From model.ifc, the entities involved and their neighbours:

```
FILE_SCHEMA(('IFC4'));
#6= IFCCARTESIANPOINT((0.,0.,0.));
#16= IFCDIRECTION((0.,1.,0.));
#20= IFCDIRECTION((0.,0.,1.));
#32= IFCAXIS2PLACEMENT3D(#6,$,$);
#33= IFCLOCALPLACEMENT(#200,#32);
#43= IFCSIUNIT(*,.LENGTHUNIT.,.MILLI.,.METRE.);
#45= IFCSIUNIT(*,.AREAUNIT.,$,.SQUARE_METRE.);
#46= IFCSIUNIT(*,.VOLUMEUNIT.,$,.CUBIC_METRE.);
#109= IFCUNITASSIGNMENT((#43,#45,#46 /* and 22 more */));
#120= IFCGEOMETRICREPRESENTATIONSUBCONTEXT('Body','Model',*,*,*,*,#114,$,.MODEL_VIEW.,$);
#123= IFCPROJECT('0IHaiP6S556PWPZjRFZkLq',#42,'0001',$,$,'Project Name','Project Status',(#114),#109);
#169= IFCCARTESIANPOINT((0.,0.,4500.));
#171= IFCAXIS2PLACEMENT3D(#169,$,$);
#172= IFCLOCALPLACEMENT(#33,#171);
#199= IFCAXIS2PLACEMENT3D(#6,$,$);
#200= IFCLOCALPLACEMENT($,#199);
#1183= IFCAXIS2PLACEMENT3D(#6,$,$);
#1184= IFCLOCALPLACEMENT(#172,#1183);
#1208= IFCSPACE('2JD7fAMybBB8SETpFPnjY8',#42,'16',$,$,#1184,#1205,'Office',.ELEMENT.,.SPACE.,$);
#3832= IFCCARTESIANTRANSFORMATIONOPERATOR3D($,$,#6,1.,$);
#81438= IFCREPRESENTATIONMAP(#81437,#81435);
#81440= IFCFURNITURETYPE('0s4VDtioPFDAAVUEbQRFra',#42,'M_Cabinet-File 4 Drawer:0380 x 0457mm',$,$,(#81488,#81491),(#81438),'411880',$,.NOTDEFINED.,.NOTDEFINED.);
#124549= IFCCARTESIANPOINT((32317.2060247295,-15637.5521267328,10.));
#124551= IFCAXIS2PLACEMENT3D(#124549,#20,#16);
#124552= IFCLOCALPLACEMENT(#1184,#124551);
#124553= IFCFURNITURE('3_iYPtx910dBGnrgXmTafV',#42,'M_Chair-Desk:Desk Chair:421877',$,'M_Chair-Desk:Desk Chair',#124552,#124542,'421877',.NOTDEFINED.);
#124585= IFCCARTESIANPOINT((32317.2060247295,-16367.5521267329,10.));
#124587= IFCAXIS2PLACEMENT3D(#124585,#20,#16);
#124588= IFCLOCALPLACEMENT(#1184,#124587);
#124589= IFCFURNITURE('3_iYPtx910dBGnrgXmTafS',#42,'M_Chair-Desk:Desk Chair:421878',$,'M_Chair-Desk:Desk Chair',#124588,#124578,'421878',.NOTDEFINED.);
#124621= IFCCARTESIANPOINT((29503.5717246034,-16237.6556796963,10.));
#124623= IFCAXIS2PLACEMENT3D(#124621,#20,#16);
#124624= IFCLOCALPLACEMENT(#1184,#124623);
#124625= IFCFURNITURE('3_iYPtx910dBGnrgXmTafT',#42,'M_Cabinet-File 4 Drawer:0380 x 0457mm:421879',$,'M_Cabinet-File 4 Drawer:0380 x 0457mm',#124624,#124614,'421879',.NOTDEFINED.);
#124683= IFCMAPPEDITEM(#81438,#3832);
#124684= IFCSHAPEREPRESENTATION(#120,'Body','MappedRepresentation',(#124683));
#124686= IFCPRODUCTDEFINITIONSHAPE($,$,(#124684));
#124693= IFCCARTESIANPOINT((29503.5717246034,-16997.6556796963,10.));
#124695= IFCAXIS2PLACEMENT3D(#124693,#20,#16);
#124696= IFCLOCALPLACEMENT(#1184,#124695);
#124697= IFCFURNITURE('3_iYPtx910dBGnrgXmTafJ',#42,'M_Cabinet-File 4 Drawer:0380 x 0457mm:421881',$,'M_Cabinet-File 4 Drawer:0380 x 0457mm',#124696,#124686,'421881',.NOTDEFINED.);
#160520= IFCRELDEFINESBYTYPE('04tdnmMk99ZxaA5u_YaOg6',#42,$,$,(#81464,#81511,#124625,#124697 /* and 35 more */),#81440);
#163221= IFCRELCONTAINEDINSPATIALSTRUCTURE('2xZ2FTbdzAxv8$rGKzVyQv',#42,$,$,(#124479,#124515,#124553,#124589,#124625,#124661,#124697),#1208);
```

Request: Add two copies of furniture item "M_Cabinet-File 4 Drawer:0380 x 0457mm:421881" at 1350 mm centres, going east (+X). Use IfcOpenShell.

```python
import numpy as np
import ifcopenshell
import ifcopenshell.api.geometry
import ifcopenshell.api.root
import ifcopenshell.util.element
import ifcopenshell.util.placement
import ifcopenshell.util.unit

model = ifcopenshell.open("model.ifc")
unit_scale = ifcopenshell.util.unit.calculate_unit_scale(model)


def reuse_history(source, copy):
    """copy_class also copies each property set's owner history, people and application; keep the originals."""
    for rel in copy.IsDefinedBy:
        if rel.is_a("IfcRelDefinesByProperties") and (history := rel.RelatingPropertyDefinition.OwnerHistory):
            rel.RelatingPropertyDefinition.OwnerHistory = source.OwnerHistory
            ifcopenshell.util.element.remove_deep2(model, history)


source = model.by_guid("3_iYPtx910dBGnrgXmTafJ")
base = ifcopenshell.util.placement.get_local_placement(source.ObjectPlacement)
step = np.array([1.0, 0.0, 0.0]) * 1.35 / unit_scale

for i in range(1, 3):
    copy = ifcopenshell.api.root.copy_class(model, product=source)
    copy.Representation = ifcopenshell.util.element.copy_deep(
        model, source.Representation, exclude=["IfcGeometricRepresentationContext", "IfcRepresentationMap"]
    )
    copy.Name = "M_Cabinet-File 4 Drawer:0380 x 0457mm"
    copy.Tag = None
    reuse_history(source, copy)
    matrix = base.copy()
    matrix[:3, 3] += i * step
    print("added at", matrix[:3, 3].round(3) + 0.0)
    ifcopenshell.api.geometry.edit_object_placement(model, product=copy, matrix=matrix, is_si=False)

model.write("model_v2.ifc")
```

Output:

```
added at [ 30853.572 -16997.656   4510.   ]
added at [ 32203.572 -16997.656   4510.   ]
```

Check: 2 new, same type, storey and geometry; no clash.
